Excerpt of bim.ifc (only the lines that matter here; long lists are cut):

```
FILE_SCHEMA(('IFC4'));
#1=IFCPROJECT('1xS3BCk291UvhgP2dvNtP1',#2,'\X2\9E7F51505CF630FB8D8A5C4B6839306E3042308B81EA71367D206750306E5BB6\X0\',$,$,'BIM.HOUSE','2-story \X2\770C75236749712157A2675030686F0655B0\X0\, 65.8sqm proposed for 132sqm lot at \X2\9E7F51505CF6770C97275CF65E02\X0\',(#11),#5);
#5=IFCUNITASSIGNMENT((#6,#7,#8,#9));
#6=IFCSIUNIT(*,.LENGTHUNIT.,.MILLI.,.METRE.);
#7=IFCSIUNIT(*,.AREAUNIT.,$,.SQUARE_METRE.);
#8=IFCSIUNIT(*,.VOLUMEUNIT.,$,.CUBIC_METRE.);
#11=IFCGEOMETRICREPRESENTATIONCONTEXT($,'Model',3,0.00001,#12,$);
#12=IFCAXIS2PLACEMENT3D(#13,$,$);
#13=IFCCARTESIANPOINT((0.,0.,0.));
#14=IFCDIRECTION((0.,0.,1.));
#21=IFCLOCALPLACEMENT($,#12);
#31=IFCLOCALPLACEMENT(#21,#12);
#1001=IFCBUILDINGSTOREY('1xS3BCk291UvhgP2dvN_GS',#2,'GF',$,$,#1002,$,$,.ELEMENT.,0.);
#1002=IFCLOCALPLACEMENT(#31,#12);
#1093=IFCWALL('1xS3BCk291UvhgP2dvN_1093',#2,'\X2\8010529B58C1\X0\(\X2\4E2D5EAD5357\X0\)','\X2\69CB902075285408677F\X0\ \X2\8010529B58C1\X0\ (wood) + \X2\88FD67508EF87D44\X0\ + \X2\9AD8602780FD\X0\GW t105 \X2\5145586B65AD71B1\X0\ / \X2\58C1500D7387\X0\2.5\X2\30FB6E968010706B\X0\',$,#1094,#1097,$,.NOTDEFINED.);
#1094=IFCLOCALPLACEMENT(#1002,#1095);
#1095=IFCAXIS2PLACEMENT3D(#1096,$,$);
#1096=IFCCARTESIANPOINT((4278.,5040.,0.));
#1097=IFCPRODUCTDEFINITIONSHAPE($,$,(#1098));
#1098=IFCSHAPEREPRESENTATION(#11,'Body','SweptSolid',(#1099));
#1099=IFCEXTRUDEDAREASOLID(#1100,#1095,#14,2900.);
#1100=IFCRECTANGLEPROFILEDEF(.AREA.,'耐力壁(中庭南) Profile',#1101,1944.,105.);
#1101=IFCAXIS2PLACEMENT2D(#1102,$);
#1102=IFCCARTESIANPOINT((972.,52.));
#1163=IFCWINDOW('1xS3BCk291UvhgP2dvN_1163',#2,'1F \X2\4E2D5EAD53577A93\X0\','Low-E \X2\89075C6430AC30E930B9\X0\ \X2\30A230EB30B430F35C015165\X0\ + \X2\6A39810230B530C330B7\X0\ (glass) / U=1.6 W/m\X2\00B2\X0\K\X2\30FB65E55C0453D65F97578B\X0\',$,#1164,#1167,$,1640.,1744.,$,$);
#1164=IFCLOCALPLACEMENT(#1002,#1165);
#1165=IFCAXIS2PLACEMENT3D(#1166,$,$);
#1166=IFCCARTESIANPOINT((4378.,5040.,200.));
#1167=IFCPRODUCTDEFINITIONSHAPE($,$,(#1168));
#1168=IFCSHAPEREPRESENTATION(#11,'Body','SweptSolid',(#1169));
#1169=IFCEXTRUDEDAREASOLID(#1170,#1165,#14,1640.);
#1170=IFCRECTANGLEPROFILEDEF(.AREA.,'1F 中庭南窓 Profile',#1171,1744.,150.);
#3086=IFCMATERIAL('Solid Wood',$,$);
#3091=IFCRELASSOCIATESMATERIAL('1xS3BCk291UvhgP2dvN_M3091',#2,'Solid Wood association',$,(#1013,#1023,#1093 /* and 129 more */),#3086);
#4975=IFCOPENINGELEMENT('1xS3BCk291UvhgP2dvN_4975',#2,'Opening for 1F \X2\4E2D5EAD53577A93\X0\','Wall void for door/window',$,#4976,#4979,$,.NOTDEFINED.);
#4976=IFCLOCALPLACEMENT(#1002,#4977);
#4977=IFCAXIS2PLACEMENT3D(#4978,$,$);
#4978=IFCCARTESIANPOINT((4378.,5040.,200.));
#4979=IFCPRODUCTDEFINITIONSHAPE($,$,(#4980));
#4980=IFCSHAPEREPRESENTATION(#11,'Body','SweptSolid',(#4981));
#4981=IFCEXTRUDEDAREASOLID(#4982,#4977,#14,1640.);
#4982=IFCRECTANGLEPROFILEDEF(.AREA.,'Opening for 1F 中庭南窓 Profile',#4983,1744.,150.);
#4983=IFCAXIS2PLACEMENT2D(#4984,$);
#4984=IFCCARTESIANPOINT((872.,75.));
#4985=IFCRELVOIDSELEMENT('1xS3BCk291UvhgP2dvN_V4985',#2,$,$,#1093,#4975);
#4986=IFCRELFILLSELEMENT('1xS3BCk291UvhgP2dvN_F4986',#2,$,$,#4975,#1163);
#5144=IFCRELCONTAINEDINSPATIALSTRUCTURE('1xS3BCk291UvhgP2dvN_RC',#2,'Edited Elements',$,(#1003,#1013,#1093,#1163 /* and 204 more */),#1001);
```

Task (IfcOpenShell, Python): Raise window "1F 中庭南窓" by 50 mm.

```python
import numpy as np
import ifcopenshell
import ifcopenshell.api.geometry
import ifcopenshell.util.placement
import ifcopenshell.util.unit

model = ifcopenshell.open("bim.ifc")
unit_scale = ifcopenshell.util.unit.calculate_unit_scale(model)

window = model.by_guid("1xS3BCk291UvhgP2dvN_1163")
opening = window.FillsVoids[0].RelatingOpeningElement
dz = 0.05 / unit_scale

shift = np.array([0.0, 0.0, dz])
# The window is not placed relative to its opening, so move both.
for product in (opening, window):
    matrix = ifcopenshell.util.placement.get_local_placement(product.ObjectPlacement)
    matrix[:3, 3] += shift
    ifcopenshell.api.geometry.edit_object_placement(model, product=product, matrix=matrix, is_si=False)

print(f"moved by {dz * unit_scale:+.3f} m")

model.write("bim_updated.ifc")
```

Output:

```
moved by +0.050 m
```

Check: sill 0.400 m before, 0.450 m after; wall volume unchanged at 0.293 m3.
